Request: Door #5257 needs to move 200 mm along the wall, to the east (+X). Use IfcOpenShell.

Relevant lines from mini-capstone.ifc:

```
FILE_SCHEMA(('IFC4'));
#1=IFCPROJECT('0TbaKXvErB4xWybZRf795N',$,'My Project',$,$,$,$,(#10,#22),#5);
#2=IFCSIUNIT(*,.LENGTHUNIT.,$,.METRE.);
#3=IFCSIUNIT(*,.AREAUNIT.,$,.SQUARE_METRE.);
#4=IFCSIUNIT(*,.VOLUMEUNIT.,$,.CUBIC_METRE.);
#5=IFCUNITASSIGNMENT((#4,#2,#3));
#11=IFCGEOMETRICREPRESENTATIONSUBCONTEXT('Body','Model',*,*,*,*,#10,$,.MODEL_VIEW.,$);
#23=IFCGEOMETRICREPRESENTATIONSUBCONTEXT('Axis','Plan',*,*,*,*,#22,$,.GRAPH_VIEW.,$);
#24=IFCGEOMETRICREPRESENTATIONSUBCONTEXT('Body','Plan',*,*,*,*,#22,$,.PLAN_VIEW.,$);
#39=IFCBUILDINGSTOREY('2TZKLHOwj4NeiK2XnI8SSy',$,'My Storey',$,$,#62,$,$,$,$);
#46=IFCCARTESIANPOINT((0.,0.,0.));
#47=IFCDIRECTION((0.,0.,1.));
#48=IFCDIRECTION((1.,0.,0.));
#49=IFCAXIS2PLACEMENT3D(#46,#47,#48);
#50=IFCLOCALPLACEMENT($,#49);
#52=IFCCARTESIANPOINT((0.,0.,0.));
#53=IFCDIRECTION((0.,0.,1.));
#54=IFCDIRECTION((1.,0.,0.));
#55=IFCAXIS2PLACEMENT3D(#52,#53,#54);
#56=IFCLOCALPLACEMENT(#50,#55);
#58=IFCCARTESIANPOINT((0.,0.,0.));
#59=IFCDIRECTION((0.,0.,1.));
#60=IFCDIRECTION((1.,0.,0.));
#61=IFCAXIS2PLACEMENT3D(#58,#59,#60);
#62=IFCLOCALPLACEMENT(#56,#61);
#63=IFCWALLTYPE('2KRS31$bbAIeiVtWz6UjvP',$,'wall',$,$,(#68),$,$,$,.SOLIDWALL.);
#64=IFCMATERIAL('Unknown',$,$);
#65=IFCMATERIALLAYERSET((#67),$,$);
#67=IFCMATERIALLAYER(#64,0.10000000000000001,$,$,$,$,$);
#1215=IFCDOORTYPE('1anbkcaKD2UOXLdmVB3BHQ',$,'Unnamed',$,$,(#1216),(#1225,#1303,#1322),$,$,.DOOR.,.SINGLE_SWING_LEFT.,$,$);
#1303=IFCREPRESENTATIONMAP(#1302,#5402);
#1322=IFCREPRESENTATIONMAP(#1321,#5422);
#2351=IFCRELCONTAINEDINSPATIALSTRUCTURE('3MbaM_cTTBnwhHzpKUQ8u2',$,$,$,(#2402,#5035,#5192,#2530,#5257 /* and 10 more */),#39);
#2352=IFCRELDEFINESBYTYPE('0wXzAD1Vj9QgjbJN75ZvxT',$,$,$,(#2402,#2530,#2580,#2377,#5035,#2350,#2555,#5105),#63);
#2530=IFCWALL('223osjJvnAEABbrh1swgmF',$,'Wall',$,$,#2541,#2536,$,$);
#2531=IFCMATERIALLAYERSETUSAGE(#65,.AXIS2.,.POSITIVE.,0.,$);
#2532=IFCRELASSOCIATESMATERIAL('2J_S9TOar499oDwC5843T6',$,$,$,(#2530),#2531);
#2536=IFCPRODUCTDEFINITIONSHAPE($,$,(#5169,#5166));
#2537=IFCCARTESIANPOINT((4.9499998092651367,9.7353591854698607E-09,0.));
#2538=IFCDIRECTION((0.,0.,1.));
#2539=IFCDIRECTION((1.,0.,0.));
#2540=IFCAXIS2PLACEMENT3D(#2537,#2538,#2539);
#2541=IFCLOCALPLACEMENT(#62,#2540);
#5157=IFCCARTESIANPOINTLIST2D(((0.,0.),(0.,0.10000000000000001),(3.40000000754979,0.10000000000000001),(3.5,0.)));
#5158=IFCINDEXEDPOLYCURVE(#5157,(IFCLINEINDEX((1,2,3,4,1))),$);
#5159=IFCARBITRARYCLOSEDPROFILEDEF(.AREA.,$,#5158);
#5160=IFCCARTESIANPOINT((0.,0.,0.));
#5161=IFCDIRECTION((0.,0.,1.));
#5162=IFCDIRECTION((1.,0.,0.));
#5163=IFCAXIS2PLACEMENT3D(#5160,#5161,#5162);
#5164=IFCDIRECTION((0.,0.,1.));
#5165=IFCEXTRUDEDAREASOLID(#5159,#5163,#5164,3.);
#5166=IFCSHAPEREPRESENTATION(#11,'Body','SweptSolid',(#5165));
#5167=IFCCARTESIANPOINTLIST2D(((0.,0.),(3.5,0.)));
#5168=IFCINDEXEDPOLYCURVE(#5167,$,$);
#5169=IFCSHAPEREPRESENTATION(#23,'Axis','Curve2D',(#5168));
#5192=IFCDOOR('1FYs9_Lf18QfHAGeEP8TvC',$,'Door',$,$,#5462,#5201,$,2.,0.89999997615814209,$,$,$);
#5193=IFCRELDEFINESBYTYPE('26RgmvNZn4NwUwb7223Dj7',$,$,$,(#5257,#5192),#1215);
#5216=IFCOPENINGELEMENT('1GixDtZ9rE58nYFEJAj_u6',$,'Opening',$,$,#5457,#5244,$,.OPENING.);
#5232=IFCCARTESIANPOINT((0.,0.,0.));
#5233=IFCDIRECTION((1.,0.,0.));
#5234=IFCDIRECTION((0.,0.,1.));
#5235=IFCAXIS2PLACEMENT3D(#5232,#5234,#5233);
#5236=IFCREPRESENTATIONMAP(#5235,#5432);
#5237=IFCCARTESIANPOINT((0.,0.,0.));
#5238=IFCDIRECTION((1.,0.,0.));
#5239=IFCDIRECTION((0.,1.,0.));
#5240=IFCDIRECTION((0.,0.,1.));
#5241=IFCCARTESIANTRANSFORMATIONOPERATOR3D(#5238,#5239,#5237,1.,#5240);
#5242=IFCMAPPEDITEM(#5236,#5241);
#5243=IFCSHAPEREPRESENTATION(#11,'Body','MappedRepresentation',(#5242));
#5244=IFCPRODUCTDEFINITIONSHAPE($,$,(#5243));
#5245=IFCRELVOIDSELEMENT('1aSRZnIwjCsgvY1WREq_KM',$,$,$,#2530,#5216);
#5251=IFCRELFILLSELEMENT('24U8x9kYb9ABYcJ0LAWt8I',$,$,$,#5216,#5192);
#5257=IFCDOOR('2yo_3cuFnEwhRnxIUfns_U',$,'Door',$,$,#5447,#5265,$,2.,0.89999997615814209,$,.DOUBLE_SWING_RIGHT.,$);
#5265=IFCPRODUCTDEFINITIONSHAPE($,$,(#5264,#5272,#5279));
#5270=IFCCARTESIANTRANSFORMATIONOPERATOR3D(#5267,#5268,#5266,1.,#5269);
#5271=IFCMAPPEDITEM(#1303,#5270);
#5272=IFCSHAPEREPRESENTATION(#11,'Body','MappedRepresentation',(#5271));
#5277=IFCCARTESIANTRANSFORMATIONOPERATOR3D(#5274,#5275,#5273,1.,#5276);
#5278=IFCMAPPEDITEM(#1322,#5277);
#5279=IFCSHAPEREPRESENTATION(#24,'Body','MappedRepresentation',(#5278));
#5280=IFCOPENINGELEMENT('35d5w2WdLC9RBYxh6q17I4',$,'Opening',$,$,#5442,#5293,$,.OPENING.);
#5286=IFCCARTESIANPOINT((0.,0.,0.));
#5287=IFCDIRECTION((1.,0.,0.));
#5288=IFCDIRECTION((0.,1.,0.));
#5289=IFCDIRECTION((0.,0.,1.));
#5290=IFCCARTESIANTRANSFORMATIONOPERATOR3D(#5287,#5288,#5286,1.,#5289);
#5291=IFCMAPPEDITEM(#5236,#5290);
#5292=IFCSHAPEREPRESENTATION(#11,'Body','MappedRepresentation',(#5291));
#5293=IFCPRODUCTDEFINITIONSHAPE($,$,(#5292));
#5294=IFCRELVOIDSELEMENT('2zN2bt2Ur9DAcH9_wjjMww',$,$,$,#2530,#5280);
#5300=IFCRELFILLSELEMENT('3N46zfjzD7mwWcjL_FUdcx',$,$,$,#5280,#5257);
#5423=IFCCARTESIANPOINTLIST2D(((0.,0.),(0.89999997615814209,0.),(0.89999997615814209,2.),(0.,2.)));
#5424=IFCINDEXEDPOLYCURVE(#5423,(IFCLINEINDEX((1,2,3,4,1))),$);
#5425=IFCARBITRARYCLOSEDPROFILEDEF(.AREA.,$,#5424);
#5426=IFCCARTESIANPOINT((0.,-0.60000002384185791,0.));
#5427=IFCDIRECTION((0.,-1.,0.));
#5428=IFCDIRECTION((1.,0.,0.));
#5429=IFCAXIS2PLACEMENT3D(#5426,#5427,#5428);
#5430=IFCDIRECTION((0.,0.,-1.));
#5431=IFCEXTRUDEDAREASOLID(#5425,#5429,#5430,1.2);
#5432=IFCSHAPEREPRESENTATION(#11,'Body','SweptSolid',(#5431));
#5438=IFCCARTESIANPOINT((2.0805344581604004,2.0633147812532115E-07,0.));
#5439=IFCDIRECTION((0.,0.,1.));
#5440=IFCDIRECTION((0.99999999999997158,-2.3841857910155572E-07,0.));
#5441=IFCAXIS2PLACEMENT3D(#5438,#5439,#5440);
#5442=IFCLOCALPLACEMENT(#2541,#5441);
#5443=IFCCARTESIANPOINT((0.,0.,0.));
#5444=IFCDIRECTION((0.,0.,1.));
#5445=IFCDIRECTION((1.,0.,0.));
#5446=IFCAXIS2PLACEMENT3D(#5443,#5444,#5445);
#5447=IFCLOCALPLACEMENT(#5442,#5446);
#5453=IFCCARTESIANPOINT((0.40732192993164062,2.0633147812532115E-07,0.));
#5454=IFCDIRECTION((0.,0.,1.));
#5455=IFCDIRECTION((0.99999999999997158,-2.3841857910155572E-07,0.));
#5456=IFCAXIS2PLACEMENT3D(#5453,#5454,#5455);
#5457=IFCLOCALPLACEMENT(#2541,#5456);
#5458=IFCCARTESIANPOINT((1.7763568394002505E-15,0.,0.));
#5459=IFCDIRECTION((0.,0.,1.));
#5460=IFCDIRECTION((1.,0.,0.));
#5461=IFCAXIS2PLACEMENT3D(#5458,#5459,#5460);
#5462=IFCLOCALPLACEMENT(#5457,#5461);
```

```python
import ifcopenshell
import ifcopenshell.api.geometry
import ifcopenshell.util.placement

model = ifcopenshell.open("mini-capstone.ifc")

door = model.by_guid("2yo_3cuFnEwhRnxIUfns_U")
opening = door.FillsVoids[0].RelatingOpeningElement
wall = opening.VoidsElements[0].RelatingBuildingElement

wall_matrix = ifcopenshell.util.placement.get_local_placement(wall.ObjectPlacement)
shift = wall_matrix[:3, 0] * 0.2
before = ifcopenshell.util.placement.get_local_placement(door.ObjectPlacement)[:3, 3].copy()

# The door is placed relative to its opening, so it follows when the opening moves.
matrix = ifcopenshell.util.placement.get_local_placement(opening.ObjectPlacement)
matrix[:3, 3] += shift
ifcopenshell.api.geometry.edit_object_placement(
    model, product=opening, matrix=matrix, is_si=False, should_transform_children=True
)

after = ifcopenshell.util.placement.get_local_placement(door.ObjectPlacement)[:3, 3]
print("door moved by", (after - before).round(3) + 0.0)

model.write("mini-capstone_edited.ifc")
```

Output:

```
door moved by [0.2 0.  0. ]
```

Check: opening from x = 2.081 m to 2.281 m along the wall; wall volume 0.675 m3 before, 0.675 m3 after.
